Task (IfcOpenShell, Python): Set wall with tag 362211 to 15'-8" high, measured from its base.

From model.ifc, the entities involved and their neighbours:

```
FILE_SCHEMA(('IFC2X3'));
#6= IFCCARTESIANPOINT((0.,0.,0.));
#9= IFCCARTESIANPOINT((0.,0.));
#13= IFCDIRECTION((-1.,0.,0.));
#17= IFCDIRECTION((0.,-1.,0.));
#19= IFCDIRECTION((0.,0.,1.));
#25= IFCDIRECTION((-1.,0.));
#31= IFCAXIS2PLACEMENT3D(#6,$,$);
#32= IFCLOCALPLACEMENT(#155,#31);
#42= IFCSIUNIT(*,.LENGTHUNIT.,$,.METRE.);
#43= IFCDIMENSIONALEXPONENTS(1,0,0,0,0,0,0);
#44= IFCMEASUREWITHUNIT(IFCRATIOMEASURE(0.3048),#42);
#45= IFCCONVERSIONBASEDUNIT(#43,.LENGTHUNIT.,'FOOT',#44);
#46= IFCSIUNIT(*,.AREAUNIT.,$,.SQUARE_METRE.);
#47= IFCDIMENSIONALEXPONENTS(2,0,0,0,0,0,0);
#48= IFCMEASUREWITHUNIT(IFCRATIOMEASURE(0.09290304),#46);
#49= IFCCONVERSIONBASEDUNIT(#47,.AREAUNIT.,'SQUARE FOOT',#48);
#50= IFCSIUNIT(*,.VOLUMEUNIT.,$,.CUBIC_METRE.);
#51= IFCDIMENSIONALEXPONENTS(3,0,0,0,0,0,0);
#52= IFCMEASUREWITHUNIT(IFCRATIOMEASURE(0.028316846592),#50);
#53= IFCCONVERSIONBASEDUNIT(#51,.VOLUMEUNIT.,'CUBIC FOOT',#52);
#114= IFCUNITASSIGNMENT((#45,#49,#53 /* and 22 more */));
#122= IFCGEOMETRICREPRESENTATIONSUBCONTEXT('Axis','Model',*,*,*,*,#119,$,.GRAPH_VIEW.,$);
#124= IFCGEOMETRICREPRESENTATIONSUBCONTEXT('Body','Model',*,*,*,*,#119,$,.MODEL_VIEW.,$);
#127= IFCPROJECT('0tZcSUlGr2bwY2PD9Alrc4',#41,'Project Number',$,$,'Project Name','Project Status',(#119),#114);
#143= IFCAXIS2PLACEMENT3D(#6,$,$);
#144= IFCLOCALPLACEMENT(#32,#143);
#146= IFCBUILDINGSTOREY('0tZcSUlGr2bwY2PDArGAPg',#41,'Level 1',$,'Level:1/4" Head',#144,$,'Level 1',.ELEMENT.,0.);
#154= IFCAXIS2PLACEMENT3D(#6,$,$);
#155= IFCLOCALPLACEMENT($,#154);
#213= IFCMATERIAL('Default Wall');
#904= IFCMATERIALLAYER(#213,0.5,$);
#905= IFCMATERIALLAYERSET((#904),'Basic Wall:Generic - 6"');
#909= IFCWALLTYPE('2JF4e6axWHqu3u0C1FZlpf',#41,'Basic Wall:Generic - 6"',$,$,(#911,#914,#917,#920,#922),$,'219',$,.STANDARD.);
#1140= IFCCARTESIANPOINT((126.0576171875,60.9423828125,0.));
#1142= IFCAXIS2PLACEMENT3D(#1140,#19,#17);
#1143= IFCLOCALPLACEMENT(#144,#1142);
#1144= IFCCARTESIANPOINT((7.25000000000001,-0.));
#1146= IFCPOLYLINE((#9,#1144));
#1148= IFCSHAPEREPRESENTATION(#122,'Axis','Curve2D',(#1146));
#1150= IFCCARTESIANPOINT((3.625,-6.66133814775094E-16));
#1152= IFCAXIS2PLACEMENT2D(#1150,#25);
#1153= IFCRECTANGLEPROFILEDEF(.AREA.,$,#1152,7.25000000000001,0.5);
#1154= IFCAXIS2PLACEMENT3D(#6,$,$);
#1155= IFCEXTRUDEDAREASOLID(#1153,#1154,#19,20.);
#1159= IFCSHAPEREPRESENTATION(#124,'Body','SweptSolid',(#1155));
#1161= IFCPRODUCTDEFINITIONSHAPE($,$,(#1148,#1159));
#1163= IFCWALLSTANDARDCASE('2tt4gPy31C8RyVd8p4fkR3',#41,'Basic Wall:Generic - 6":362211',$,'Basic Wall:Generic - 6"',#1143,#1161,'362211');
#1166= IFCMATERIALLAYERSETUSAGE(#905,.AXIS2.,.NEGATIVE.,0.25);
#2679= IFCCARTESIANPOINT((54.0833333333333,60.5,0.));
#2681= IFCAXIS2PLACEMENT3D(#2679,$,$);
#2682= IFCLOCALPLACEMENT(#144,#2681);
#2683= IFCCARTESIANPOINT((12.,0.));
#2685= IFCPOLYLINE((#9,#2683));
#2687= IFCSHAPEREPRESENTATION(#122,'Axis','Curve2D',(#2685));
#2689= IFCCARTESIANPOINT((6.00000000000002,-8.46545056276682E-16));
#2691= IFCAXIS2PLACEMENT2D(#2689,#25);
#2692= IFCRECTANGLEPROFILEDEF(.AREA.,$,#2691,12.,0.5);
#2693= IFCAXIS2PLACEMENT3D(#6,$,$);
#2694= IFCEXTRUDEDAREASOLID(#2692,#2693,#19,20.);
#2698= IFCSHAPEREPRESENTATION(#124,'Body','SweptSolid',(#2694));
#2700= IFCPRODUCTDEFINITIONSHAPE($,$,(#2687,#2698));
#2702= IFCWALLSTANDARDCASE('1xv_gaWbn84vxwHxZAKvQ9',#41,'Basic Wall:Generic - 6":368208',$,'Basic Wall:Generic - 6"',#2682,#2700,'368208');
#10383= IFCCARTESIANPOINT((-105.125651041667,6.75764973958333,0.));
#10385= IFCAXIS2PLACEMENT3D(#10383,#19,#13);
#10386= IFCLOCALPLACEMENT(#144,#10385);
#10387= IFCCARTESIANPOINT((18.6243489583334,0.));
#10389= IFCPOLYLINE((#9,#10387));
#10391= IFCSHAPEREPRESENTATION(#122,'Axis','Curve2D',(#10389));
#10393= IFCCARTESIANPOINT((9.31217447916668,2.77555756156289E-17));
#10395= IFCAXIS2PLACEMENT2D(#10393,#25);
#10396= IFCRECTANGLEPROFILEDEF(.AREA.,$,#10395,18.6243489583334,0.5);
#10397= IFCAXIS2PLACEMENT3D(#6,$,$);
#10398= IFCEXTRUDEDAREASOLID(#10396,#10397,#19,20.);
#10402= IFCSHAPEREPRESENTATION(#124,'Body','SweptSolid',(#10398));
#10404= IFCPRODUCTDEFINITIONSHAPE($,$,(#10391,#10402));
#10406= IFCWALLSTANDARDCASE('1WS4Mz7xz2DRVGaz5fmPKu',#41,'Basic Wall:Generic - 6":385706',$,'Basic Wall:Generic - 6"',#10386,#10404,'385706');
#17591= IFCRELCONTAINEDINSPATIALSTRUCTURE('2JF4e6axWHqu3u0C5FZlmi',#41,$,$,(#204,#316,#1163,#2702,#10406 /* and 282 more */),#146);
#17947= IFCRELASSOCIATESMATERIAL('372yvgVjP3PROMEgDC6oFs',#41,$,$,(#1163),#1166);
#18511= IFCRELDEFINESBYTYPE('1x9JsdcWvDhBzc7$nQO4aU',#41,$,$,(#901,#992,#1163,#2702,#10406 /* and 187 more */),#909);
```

```python
import ifcopenshell
import ifcopenshell.geom
import ifcopenshell.util.representation
import ifcopenshell.util.shape
import ifcopenshell.util.unit

model = ifcopenshell.open("model.ifc")
unit_scale = ifcopenshell.util.unit.calculate_unit_scale(model)
settings = ifcopenshell.geom.settings()


def volume(element):
    """Net volume in cubic metres, openings subtracted."""
    shape = ifcopenshell.geom.create_shape(settings, element)
    return ifcopenshell.util.shape.get_volume(shape.geometry)


wall = model.by_guid("2tt4gPy31C8RyVd8p4fkR3")
before = volume(wall)

body = ifcopenshell.util.representation.get_representation(wall, "Model", "Body")
solid = body.Items[0]
old_height = solid.Depth
solid.Depth = 188 * 0.0254 / unit_scale
after = volume(wall)

print(f"height {old_height:g} -> {solid.Depth:g}, volume {before:.3f} -> {after:.3f} m3")

model.write("model_rev.ifc")
```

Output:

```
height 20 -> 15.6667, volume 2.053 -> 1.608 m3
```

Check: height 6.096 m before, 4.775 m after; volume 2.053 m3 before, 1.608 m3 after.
